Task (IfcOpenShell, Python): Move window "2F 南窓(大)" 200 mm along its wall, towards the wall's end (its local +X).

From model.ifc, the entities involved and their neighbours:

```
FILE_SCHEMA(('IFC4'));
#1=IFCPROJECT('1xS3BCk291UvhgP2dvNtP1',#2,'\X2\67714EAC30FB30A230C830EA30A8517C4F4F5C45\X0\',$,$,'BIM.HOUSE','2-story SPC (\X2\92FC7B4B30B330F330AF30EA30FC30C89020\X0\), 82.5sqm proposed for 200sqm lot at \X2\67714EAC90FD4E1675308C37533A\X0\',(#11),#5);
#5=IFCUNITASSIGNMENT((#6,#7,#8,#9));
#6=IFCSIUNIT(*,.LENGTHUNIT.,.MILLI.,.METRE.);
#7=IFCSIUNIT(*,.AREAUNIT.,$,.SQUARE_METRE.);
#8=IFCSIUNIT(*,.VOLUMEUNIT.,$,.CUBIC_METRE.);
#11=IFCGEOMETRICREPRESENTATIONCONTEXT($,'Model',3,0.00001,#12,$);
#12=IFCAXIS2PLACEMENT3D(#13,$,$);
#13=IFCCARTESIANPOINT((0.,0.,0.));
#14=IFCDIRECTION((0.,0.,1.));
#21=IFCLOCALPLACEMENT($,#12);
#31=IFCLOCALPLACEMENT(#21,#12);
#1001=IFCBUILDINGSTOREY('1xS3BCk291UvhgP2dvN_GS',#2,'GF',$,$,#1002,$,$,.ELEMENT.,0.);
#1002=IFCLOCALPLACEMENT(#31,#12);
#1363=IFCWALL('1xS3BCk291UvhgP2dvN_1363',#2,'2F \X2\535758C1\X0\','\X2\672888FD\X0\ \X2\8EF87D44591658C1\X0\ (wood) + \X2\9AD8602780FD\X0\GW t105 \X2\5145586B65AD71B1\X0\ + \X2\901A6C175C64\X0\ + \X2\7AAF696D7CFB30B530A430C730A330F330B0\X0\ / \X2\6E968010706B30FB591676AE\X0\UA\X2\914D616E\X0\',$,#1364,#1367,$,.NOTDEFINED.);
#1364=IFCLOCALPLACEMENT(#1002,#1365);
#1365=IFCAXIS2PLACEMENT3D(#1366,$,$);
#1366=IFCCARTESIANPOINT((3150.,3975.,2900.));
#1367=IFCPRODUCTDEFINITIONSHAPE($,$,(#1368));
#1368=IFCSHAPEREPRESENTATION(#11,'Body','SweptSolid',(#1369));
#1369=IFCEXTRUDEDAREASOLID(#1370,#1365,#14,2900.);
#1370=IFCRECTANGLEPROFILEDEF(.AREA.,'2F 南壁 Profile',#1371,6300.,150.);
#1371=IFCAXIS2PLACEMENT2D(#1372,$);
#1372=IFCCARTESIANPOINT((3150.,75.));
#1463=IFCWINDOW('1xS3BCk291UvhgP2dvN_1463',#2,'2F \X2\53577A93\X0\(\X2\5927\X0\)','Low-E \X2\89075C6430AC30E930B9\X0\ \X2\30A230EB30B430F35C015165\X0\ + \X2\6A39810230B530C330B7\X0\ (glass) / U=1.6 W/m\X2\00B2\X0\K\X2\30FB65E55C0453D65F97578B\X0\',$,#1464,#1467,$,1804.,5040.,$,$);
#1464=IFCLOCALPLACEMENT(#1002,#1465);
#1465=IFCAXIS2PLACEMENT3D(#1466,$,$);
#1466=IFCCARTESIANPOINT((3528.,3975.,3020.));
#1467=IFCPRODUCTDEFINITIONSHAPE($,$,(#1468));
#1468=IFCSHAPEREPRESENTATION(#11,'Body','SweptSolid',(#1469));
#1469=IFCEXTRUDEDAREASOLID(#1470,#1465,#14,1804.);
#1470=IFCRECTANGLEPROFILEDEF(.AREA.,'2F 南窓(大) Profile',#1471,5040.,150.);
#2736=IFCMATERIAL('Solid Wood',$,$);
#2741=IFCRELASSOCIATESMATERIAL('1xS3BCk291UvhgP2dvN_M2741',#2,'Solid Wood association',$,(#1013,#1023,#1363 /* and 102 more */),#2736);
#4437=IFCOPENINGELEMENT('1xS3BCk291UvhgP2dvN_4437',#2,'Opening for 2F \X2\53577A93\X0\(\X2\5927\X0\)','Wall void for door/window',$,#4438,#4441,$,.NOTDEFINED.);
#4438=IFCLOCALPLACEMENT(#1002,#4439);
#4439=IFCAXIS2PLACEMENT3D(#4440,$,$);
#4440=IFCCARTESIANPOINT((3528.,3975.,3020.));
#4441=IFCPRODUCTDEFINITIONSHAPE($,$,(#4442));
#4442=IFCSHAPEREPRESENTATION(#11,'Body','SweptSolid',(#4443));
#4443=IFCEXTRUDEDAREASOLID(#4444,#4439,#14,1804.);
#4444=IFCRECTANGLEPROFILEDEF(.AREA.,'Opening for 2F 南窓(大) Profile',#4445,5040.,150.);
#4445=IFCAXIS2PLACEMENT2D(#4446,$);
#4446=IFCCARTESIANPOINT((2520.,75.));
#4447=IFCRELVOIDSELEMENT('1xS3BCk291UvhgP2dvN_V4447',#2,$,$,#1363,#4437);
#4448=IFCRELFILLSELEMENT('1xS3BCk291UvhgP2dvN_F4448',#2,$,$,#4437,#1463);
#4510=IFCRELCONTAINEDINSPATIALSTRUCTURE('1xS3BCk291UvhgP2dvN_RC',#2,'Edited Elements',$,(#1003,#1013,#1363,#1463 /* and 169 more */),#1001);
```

```python
import ifcopenshell
import ifcopenshell.api.geometry
import ifcopenshell.util.placement
import ifcopenshell.util.unit

model = ifcopenshell.open("model.ifc")
unit_scale = ifcopenshell.util.unit.calculate_unit_scale(model)

window = model.by_guid("1xS3BCk291UvhgP2dvN_1463")
opening = window.FillsVoids[0].RelatingOpeningElement
wall = opening.VoidsElements[0].RelatingBuildingElement

wall_matrix = ifcopenshell.util.placement.get_local_placement(wall.ObjectPlacement)
shift = wall_matrix[:3, 0] * 0.2 / unit_scale
before = ifcopenshell.util.placement.get_local_placement(window.ObjectPlacement)[:3, 3].copy()

# The window is not placed relative to its opening, so move both.
for product in (opening, window):
    matrix = ifcopenshell.util.placement.get_local_placement(product.ObjectPlacement)
    matrix[:3, 3] += shift
    ifcopenshell.api.geometry.edit_object_placement(model, product=product, matrix=matrix, is_si=False)

after = ifcopenshell.util.placement.get_local_placement(window.ObjectPlacement)[:3, 3]
print("window moved by", (after - before).round(3) + 0.0)

model.write("model_edited.ifc")
```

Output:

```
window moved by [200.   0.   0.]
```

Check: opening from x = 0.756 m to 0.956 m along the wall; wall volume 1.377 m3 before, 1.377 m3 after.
